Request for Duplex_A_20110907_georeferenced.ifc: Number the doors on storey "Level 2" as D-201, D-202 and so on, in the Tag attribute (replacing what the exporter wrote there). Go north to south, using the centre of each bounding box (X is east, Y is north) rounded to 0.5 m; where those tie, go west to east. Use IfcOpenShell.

First a look at what the model holds.

```python
import ifcopenshell
import ifcopenshell.util.element
import ifcopenshell.util.placement

model = ifcopenshell.open("Duplex_A_20110907_georeferenced.ifc")
print(model.schema)
storey = next(s for s in model.by_type("IfcBuildingStorey") if s.Name == "Level 2")
doors = [e for e in ifcopenshell.util.element.get_decomposition(storey) if e.is_a("IfcDoor")]
for e in sorted(doors, key=lambda e: e.id()):
    origin = ifcopenshell.util.placement.get_local_placement(e.ObjectPlacement)[:3, 3]
    print(e.id(), e.Tag, e.Name, origin.round(2) + 0.0, sep=" | ")
```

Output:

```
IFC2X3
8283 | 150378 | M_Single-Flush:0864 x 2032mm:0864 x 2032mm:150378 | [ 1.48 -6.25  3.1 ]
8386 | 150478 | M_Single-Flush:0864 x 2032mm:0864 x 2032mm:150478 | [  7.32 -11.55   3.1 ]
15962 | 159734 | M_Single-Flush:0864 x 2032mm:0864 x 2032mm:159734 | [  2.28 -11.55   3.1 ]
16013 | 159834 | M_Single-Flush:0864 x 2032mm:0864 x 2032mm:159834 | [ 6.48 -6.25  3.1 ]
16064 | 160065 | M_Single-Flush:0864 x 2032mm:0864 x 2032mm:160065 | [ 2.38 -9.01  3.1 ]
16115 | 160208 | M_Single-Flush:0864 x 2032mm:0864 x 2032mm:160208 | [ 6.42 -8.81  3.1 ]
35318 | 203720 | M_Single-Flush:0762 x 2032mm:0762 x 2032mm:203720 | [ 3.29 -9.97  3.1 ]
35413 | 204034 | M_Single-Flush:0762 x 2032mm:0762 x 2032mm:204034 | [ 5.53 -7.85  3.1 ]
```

```python
import ifcopenshell
import ifcopenshell.geom
import ifcopenshell.util.element
import ifcopenshell.util.shape

model = ifcopenshell.open("Duplex_A_20110907_georeferenced.ifc")
settings = ifcopenshell.geom.settings()
settings.set("use-world-coords", True)


def centre(element):
    shape = ifcopenshell.geom.create_shape(settings, element)
    return ifcopenshell.util.shape.get_bbox_centroid(shape.geometry)


storey = next(s for s in model.by_type("IfcBuildingStorey") if s.Name == "Level 2")
doors = [e for e in ifcopenshell.util.element.get_decomposition(storey) if e.is_a("IfcDoor")]

# Insertion points can sit at a corner or the storey origin, so sort by the geometry (in metres).
centres = {e: centre(e) for e in doors}
doors.sort(key=lambda e: (-round(centres[e][1] / 0.5), centres[e][0]))

for i, e in enumerate(doors, start=1):
    number = f"D-2{i:02d}"
    e.Tag = number
    print(e.id(), number)

model.write("Duplex_A_20110907_georeferenced_rev.ifc")
```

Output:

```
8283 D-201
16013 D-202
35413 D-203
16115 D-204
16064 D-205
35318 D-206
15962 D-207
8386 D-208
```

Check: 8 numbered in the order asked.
